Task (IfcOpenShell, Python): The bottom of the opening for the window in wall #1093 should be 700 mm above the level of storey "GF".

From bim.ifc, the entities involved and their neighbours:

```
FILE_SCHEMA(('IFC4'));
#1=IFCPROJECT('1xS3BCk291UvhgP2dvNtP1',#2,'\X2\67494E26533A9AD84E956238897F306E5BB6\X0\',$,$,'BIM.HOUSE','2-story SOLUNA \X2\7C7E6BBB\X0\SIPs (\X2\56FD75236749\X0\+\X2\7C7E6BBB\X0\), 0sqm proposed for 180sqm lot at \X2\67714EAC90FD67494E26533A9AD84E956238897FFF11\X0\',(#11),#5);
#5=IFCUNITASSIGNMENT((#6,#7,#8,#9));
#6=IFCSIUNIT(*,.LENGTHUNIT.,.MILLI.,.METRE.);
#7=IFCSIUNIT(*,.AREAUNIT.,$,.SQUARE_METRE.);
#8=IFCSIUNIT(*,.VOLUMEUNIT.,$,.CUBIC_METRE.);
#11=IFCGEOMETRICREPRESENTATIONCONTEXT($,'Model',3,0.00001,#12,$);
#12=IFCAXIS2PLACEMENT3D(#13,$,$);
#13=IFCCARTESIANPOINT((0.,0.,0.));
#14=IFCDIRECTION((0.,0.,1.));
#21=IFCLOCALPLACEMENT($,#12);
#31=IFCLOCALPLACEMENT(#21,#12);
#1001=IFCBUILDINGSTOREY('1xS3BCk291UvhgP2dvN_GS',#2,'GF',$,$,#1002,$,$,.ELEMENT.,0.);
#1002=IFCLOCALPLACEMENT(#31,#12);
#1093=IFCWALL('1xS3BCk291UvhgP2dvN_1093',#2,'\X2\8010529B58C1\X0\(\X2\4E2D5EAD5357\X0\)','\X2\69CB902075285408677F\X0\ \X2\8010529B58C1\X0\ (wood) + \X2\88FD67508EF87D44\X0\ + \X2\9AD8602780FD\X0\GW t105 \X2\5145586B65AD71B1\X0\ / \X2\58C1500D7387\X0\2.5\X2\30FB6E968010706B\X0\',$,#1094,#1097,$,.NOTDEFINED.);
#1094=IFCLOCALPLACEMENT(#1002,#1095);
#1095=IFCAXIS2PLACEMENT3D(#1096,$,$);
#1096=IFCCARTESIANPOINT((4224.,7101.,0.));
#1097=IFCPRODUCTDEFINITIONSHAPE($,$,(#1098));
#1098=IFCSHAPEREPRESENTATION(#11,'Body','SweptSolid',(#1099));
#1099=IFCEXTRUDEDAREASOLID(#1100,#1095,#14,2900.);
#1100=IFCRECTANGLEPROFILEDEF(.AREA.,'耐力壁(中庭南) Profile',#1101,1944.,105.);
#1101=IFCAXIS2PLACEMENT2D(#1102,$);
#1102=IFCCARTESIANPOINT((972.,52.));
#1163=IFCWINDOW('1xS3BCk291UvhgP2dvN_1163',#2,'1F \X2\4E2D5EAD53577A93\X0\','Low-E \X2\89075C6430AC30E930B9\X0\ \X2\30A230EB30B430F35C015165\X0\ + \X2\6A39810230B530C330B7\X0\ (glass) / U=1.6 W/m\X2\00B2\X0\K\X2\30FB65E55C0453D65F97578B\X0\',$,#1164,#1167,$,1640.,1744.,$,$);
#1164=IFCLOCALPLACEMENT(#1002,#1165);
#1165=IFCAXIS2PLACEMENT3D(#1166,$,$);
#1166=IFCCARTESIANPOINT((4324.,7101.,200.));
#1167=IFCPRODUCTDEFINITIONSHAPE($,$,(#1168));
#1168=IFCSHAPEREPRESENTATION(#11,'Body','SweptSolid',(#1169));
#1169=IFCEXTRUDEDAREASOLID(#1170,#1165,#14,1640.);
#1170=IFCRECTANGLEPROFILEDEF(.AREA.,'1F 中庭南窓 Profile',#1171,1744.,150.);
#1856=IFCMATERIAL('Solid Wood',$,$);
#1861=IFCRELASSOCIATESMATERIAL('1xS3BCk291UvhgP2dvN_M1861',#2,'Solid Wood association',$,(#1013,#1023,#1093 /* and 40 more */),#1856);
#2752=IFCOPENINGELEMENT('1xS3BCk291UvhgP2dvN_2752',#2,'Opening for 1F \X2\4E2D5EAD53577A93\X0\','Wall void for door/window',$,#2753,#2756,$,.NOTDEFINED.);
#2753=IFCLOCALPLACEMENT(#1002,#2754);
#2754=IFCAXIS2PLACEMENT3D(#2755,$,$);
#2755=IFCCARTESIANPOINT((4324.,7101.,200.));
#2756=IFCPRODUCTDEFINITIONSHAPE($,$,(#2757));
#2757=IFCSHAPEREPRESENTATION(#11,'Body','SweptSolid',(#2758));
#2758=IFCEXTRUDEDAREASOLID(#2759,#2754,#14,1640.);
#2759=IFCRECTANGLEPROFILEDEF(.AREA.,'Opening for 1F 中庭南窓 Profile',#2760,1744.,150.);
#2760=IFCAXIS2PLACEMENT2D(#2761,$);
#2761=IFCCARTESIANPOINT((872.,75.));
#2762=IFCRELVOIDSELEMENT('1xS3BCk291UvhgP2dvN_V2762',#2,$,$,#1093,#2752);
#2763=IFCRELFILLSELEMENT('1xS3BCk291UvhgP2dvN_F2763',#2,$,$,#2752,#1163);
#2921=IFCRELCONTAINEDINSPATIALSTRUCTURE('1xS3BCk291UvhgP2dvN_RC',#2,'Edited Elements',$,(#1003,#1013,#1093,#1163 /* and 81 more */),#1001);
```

```python
import numpy as np
import ifcopenshell
import ifcopenshell.api.geometry
import ifcopenshell.geom
import ifcopenshell.util.element
import ifcopenshell.util.placement
import ifcopenshell.util.shape
import ifcopenshell.util.unit

model = ifcopenshell.open("bim.ifc")
unit_scale = ifcopenshell.util.unit.calculate_unit_scale(model)

window = model.by_id(1163)
opening = window.FillsVoids[0].RelatingOpeningElement
storey = ifcopenshell.util.element.get_container(window, ifc_class="IfcBuildingStorey")
level = ifcopenshell.util.placement.get_local_placement(storey.ObjectPlacement)[2, 3]

# The opening's origin need not be at the sill, so measure its lowest point.
shape = ifcopenshell.geom.create_shape(ifcopenshell.geom.settings(), opening)
bottom = ifcopenshell.util.shape.get_shape_bottom_elevation(shape, shape.geometry) / unit_scale
dz = level + 700.0 - bottom

shift = np.array([0.0, 0.0, dz])
# The window is not placed relative to its opening, so move both.
for product in (opening, window):
    matrix = ifcopenshell.util.placement.get_local_placement(product.ObjectPlacement)
    matrix[:3, 3] += shift
    ifcopenshell.api.geometry.edit_object_placement(model, product=product, matrix=matrix, is_si=False)

print(f"moved by {dz * unit_scale:+.3f} m")

model.write("bim_rev.ifc")
```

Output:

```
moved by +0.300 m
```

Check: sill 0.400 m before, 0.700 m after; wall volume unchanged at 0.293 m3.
